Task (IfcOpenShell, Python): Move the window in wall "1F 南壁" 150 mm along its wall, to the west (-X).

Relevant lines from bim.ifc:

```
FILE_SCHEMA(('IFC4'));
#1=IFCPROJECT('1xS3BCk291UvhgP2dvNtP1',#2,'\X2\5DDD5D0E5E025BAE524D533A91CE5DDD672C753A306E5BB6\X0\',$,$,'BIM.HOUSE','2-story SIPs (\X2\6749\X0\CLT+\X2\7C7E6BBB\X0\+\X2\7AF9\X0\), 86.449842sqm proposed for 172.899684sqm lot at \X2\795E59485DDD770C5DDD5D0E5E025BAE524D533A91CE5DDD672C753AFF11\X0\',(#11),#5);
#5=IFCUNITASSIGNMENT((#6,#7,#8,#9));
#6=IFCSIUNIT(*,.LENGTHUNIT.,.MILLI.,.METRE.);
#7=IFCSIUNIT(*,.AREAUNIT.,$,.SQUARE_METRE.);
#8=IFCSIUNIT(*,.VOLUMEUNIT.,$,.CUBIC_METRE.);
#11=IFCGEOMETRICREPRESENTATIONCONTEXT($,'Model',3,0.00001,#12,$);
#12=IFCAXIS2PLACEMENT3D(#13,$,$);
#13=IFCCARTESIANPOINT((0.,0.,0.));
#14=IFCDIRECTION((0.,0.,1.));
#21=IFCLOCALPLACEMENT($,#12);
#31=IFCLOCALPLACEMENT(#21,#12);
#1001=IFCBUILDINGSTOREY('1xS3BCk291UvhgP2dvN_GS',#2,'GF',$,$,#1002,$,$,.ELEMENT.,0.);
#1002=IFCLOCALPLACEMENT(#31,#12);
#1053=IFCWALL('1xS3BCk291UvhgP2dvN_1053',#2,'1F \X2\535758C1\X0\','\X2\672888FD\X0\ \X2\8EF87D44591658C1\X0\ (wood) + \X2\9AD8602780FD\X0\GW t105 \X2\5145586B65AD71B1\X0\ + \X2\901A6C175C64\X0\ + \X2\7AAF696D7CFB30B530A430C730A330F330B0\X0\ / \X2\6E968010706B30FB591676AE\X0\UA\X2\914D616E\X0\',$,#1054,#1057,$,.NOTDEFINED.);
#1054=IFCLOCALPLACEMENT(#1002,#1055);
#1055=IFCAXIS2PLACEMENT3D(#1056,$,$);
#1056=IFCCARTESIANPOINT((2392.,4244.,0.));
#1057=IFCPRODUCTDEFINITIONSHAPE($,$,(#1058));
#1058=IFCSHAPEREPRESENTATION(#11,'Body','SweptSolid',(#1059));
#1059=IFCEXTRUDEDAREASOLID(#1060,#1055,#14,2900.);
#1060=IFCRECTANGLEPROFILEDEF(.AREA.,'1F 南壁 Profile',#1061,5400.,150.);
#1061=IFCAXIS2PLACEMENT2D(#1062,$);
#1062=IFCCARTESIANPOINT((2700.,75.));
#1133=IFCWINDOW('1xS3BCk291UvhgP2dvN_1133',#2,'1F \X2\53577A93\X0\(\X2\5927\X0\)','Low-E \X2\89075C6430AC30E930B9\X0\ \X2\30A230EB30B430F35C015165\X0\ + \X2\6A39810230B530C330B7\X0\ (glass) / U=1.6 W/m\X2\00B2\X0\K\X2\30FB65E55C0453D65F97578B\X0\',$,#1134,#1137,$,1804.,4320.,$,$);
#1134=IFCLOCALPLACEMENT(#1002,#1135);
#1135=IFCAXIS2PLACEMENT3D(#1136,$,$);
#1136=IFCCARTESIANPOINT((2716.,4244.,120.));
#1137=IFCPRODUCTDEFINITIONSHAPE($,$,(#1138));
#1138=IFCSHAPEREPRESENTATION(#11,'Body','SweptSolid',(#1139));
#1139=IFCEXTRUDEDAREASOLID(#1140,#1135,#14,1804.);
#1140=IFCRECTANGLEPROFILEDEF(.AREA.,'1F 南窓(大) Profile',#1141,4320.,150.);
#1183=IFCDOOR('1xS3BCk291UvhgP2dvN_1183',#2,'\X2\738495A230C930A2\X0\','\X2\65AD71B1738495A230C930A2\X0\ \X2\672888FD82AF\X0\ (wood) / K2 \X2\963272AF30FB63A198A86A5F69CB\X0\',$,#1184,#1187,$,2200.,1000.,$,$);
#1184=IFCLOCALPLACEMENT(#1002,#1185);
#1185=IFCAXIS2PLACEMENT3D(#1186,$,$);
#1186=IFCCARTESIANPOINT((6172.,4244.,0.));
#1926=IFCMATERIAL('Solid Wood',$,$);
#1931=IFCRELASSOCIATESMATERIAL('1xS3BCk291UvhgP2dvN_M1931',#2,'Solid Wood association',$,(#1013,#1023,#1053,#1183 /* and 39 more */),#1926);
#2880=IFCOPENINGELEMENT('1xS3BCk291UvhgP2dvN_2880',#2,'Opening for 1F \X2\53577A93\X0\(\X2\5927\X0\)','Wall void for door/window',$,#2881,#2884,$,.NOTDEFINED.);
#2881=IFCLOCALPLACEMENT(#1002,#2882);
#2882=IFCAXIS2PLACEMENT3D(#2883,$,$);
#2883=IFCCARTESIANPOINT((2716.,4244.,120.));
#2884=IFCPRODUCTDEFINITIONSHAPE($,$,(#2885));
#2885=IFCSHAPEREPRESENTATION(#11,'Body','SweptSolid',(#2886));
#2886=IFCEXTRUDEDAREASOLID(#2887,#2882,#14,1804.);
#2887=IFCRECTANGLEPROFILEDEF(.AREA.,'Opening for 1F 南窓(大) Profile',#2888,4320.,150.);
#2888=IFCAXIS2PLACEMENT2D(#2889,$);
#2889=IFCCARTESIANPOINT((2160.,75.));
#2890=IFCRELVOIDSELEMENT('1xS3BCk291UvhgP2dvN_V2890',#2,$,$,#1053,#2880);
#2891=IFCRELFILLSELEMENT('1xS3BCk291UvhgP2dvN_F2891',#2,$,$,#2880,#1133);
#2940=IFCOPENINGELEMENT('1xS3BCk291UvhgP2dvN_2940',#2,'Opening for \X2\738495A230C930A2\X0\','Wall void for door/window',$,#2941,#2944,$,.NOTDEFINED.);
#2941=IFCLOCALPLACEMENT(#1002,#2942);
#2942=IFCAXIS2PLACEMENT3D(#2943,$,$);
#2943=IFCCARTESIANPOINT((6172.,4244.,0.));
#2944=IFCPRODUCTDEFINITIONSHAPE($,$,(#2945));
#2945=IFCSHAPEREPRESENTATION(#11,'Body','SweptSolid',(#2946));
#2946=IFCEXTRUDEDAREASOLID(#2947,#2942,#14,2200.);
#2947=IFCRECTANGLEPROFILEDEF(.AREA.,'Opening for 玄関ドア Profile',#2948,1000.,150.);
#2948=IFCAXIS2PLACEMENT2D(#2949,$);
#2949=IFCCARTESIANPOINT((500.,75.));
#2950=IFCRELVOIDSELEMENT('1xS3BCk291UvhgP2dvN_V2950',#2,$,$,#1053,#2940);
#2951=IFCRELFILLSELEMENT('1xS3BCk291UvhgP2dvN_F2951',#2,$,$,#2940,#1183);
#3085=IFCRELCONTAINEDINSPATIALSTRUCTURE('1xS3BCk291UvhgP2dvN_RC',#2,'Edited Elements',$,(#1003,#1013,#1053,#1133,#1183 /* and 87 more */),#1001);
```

```python
import ifcopenshell
import ifcopenshell.api.geometry
import ifcopenshell.util.placement
import ifcopenshell.util.unit

model = ifcopenshell.open("bim.ifc")
unit_scale = ifcopenshell.util.unit.calculate_unit_scale(model)

window = model.by_guid("1xS3BCk291UvhgP2dvN_1133")
opening = window.FillsVoids[0].RelatingOpeningElement
wall = opening.VoidsElements[0].RelatingBuildingElement

wall_matrix = ifcopenshell.util.placement.get_local_placement(wall.ObjectPlacement)
shift = wall_matrix[:3, 0] * -0.15 / unit_scale
before = ifcopenshell.util.placement.get_local_placement(window.ObjectPlacement)[:3, 3].copy()

# The window is not placed relative to its opening, so move both.
for product in (opening, window):
    matrix = ifcopenshell.util.placement.get_local_placement(product.ObjectPlacement)
    matrix[:3, 3] += shift
    ifcopenshell.api.geometry.edit_object_placement(model, product=product, matrix=matrix, is_si=False)

after = ifcopenshell.util.placement.get_local_placement(window.ObjectPlacement)[:3, 3]
print("window moved by", (after - before).round(3) + 0.0)

model.write("bim-out.ifc")
```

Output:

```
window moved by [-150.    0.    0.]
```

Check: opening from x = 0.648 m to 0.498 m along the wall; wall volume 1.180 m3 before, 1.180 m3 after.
